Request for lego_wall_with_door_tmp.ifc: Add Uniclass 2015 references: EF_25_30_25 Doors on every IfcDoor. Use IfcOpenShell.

First a look at what the model holds.

```python
import ifcopenshell

model = ifcopenshell.open("lego_wall_with_door_tmp.ifc")
print(model.schema)
print("classifications:", [c.Name for c in model.by_type("IfcClassification")])
for ifc_class in ("IfcDoor", "IfcRoof", "IfcStair", "IfcWall", "IfcWindow"):
    print(ifc_class, len(model.by_type(ifc_class)))
```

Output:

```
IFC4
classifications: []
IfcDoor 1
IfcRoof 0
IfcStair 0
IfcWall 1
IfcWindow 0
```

```python
import ifcopenshell
import ifcopenshell.api.classification

model = ifcopenshell.open("lego_wall_with_door_tmp.ifc")

system = ifcopenshell.api.classification.add_classification(model, classification="Uniclass 2015")

codes = {
    "IfcDoor": ("EF_25_30_25", "Doors"),
}
for ifc_class, (code, name) in codes.items():
    products = model.by_type(ifc_class)
    ifcopenshell.api.classification.add_reference(
        model, products=products, classification=system, identification=code, name=name
    )
    print(code, len(products))

model.write("lego_wall_with_door_tmp_rev.ifc")
```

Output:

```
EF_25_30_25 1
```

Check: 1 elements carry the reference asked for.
